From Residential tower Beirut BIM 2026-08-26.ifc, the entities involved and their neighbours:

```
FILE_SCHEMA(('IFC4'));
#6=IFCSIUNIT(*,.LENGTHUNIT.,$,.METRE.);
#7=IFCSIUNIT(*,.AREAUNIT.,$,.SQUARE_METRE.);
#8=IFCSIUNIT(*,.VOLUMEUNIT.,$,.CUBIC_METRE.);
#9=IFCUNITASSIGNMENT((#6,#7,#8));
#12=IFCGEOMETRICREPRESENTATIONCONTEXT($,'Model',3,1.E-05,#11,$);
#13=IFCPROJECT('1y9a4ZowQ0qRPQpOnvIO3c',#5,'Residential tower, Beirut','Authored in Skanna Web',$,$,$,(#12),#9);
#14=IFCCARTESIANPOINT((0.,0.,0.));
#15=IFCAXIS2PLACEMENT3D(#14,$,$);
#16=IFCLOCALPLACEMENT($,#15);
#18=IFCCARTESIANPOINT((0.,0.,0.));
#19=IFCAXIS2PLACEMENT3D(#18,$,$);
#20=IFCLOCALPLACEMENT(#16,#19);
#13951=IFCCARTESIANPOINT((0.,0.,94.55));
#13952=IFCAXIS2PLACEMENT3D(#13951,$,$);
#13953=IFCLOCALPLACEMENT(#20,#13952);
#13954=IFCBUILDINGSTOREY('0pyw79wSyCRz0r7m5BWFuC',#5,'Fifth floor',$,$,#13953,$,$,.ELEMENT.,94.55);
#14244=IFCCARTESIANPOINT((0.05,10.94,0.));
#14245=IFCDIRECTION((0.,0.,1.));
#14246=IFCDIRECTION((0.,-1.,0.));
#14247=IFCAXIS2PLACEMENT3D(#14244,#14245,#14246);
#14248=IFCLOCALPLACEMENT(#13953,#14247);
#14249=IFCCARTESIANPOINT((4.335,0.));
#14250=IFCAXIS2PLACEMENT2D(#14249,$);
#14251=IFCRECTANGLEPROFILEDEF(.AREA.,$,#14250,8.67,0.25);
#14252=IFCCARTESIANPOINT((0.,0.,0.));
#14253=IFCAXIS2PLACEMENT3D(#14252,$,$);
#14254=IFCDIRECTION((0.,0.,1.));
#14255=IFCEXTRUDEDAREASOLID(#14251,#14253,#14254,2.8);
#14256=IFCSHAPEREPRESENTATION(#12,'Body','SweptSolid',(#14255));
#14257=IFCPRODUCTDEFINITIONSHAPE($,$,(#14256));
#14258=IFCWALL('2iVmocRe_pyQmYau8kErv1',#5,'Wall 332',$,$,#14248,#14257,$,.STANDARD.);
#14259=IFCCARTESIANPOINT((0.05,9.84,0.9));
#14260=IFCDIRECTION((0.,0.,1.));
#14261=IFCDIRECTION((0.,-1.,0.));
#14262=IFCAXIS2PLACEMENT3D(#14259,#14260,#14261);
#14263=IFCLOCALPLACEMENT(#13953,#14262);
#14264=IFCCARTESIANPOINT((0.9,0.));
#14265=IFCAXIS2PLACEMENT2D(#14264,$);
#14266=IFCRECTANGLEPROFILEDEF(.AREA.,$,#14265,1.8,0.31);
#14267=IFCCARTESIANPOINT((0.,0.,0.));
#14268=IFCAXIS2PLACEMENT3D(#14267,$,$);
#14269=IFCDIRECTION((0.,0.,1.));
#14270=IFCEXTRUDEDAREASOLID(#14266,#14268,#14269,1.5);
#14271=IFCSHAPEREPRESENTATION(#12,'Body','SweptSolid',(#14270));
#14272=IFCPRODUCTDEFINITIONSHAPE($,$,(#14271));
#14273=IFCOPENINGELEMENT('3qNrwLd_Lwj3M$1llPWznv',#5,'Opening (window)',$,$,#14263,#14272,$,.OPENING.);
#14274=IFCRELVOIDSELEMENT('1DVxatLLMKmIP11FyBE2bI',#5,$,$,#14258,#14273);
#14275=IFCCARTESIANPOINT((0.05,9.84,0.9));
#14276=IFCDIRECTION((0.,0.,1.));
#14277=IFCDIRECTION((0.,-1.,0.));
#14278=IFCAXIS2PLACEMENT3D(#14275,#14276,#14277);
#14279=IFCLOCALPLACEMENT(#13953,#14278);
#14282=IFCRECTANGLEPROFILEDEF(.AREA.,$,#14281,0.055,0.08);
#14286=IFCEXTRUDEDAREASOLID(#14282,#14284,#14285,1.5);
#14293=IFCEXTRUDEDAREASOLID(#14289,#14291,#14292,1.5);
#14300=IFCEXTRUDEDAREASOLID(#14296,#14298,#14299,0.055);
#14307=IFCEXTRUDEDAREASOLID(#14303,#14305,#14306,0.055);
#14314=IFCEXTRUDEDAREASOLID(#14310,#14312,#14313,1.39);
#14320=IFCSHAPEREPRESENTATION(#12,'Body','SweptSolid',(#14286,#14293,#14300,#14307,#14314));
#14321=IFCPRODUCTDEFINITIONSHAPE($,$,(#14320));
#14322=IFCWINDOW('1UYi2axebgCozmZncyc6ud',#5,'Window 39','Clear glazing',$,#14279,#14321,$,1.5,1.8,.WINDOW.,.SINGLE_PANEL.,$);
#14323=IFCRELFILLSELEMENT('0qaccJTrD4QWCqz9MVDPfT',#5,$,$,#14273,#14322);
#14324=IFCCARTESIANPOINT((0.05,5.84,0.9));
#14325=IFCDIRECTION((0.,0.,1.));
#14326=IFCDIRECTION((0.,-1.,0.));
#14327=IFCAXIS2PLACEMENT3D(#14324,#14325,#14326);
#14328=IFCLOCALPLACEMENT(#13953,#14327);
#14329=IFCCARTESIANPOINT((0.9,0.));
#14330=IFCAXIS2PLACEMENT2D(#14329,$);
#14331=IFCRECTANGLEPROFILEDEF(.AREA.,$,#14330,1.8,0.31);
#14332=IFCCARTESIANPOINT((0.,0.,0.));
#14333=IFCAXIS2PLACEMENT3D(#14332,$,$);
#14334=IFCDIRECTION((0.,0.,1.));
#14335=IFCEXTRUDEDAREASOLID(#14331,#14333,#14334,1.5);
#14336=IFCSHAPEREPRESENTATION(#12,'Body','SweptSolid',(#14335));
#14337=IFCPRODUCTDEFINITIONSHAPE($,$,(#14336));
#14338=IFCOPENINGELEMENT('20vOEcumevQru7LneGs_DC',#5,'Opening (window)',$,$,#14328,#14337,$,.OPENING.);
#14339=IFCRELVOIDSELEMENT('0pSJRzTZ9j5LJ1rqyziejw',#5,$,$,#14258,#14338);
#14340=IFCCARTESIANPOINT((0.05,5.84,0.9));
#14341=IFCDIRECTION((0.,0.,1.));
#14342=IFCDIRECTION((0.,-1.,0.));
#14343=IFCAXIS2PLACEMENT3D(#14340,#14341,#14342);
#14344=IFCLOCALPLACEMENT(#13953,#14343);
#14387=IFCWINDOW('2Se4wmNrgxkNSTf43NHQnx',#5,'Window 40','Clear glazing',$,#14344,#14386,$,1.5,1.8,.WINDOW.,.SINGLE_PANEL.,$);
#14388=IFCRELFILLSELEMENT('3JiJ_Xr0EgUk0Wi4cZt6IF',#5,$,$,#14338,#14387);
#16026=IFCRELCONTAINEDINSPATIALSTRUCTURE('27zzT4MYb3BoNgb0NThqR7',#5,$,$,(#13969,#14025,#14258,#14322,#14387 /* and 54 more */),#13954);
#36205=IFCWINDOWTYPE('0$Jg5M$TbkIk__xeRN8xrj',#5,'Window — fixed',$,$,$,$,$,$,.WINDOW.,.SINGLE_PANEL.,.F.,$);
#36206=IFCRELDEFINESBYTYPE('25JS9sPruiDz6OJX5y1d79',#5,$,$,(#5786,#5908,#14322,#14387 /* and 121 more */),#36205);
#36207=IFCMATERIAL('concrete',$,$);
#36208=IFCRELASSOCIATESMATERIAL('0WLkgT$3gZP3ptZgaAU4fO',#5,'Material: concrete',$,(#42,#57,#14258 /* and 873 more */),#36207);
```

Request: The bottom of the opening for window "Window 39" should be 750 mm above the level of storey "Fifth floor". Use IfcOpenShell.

```python
import numpy as np
import ifcopenshell
import ifcopenshell.api.geometry
import ifcopenshell.geom
import ifcopenshell.util.element
import ifcopenshell.util.placement
import ifcopenshell.util.shape
import ifcopenshell.util.unit

model = ifcopenshell.open("Residential tower Beirut BIM 2026-08-26.ifc")
unit_scale = ifcopenshell.util.unit.calculate_unit_scale(model)

window = model.by_id(14322)
opening = window.FillsVoids[0].RelatingOpeningElement
storey = ifcopenshell.util.element.get_container(window, ifc_class="IfcBuildingStorey")
level = ifcopenshell.util.placement.get_local_placement(storey.ObjectPlacement)[2, 3]

# The opening's origin need not be at the sill, so measure its lowest point.
shape = ifcopenshell.geom.create_shape(ifcopenshell.geom.settings(), opening)
bottom = ifcopenshell.util.shape.get_shape_bottom_elevation(shape, shape.geometry) / unit_scale
dz = level + 0.75 / unit_scale - bottom

shift = np.array([0.0, 0.0, dz])
# The window is not placed relative to its opening, so move both.
for product in (opening, window):
    matrix = ifcopenshell.util.placement.get_local_placement(product.ObjectPlacement)
    matrix[:3, 3] += shift
    ifcopenshell.api.geometry.edit_object_placement(model, product=product, matrix=matrix, is_si=False)

print(f"moved by {dz * unit_scale:+.3f} m")

model.write("Residential tower Beirut BIM 2026-08-26_updated.ifc")
```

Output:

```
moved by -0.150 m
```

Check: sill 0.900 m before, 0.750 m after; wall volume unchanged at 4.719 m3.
